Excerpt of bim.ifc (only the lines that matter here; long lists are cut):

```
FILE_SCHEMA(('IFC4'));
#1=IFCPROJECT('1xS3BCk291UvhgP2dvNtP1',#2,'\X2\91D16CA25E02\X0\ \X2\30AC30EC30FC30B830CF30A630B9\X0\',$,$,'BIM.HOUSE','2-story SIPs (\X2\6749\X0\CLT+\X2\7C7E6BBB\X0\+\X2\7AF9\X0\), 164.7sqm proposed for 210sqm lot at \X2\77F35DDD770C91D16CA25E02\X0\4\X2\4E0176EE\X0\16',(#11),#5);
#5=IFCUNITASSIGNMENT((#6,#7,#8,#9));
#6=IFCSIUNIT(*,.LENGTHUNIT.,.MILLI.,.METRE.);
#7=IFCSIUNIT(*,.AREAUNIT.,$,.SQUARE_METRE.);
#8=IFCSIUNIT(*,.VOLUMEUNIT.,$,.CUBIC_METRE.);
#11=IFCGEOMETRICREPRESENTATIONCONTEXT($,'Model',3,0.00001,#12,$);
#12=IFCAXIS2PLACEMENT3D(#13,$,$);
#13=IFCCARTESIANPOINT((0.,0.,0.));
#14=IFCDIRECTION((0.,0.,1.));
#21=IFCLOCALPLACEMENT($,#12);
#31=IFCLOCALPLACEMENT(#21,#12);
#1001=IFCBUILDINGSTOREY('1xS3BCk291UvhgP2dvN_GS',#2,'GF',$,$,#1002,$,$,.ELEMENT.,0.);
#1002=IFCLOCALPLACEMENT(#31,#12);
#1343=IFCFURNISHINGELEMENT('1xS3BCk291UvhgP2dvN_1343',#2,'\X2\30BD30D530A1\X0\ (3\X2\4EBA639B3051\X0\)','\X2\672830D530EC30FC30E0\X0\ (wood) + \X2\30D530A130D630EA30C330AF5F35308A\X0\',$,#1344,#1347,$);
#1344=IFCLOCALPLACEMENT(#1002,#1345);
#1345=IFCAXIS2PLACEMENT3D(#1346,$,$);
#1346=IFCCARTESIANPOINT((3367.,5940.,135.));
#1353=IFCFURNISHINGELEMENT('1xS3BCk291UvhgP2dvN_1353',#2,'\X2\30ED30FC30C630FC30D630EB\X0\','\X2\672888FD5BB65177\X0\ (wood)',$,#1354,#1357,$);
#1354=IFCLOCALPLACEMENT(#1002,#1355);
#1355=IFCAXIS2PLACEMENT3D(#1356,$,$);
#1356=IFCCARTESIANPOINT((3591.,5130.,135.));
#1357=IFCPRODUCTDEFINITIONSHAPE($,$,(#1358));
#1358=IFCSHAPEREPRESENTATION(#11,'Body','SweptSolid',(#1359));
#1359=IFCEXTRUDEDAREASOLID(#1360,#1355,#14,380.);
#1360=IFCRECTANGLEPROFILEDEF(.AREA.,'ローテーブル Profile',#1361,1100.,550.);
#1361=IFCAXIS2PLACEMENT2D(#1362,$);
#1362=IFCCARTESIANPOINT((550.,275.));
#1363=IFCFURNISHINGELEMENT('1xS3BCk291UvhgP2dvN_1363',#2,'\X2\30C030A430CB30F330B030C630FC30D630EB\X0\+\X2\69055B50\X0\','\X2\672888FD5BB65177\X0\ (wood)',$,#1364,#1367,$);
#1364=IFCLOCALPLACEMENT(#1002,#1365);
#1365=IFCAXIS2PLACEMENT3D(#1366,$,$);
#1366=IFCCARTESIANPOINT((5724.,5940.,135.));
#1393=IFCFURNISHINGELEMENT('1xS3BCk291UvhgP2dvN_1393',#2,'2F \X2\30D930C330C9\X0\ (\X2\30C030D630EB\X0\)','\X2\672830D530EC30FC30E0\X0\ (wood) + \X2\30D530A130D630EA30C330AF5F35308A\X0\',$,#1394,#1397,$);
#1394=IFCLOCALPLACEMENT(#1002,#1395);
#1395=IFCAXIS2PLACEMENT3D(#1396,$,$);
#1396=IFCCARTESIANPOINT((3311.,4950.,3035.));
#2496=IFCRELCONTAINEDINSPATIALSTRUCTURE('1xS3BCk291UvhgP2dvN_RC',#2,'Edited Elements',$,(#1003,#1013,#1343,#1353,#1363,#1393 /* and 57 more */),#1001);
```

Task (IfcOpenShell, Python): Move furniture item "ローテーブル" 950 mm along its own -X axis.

```python
import ifcopenshell
import ifcopenshell.api.geometry
import ifcopenshell.util.placement
import ifcopenshell.util.unit

model = ifcopenshell.open("bim.ifc")
unit_scale = ifcopenshell.util.unit.calculate_unit_scale(model)

item = model.by_guid("1xS3BCk291UvhgP2dvN_1353")
matrix = ifcopenshell.util.placement.get_local_placement(item.ObjectPlacement)
matrix[:3, 3] -= matrix[:3, 0] * 0.95 / unit_scale
ifcopenshell.api.geometry.edit_object_placement(model, product=item, matrix=matrix, is_si=False)

print(ifcopenshell.util.placement.get_local_placement(item.ObjectPlacement).round(3) + 0.0)

model.write("bim_updated.ifc")
```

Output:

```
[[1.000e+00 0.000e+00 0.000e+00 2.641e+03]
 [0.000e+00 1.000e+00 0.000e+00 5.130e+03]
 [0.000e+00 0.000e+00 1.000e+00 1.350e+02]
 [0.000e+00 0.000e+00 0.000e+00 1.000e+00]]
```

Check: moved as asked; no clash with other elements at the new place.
